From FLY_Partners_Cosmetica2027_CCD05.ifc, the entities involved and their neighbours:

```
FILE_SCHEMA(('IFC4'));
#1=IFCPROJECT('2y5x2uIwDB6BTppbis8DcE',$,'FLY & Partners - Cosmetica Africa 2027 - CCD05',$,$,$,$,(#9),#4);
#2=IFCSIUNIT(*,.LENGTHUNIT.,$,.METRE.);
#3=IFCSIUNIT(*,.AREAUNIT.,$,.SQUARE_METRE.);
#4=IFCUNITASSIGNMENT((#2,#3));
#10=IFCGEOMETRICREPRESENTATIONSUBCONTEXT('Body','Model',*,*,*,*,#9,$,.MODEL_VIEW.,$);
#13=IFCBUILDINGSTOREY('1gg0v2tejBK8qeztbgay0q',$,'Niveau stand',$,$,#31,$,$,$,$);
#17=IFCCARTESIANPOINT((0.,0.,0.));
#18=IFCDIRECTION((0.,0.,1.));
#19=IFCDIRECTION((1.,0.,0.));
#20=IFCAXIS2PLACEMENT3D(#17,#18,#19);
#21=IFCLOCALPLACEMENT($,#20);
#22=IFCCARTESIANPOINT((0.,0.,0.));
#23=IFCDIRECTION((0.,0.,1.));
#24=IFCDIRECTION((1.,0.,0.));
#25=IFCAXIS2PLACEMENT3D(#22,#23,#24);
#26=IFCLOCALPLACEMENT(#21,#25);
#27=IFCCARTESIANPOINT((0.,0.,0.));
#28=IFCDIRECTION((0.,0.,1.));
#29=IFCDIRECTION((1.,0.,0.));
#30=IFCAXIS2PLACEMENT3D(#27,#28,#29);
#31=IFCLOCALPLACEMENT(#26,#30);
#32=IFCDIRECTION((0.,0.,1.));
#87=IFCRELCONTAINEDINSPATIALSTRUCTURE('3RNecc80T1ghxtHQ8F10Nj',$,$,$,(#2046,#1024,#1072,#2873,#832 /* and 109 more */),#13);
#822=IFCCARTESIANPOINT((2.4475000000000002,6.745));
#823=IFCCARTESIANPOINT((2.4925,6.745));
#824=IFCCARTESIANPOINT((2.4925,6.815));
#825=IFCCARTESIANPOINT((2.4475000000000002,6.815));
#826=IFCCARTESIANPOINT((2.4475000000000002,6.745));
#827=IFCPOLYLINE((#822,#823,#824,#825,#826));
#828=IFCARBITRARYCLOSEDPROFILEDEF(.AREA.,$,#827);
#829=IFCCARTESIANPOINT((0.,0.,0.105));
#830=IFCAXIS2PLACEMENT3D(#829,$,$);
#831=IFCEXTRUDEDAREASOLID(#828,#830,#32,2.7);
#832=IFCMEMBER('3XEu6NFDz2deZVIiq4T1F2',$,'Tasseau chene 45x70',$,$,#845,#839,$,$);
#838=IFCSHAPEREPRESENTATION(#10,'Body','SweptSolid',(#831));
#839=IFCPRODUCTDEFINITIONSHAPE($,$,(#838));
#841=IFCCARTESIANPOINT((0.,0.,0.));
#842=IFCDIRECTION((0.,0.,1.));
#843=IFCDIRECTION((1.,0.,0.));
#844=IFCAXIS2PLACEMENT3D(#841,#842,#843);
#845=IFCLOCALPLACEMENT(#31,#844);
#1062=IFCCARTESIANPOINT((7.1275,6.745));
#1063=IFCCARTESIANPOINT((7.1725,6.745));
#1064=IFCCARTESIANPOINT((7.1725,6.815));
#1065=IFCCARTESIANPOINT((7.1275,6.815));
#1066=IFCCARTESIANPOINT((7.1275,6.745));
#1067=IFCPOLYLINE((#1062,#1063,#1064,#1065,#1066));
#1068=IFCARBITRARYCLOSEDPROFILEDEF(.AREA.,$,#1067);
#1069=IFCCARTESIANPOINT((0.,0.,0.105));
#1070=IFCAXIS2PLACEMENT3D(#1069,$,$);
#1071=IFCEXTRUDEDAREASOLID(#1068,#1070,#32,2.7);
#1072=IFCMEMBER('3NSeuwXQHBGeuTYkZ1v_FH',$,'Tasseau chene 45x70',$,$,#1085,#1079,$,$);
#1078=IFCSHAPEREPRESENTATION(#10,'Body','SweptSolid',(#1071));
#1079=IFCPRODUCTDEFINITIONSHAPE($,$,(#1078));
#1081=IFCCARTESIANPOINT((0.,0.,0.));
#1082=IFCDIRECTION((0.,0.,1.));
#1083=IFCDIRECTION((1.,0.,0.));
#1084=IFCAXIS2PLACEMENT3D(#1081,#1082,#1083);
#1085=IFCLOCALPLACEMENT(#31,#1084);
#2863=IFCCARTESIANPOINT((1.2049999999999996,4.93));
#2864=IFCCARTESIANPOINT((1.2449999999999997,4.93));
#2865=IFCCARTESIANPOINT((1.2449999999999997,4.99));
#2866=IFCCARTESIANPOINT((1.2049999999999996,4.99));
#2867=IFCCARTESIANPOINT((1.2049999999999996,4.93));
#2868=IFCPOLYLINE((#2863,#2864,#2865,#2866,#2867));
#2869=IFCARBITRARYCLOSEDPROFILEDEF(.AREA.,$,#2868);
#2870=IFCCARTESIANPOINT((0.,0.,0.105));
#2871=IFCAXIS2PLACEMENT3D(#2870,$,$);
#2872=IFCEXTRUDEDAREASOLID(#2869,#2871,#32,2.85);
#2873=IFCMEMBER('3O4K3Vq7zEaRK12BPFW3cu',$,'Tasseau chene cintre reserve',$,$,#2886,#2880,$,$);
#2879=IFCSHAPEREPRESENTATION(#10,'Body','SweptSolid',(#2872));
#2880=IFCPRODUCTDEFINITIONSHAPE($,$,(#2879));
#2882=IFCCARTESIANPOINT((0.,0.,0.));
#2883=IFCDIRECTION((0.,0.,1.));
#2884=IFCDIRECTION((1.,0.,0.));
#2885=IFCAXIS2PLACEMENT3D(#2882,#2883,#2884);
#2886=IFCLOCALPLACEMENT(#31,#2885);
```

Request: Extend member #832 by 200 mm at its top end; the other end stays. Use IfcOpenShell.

```python
import ifcopenshell
import ifcopenshell.util.representation
import ifcopenshell.util.unit

model = ifcopenshell.open("FLY_Partners_Cosmetica2027_CCD05.ifc")
unit_scale = ifcopenshell.util.unit.calculate_unit_scale(model)

member = model.by_guid("3XEu6NFDz2deZVIiq4T1F2")
change = 0.2 / unit_scale

# The extrusion runs towards the end named, so only its depth changes.
body = ifcopenshell.util.representation.get_representation(member, "Model", "Body")
solid = body.Items[0]
old_length = solid.Depth
solid.Depth += change

print(f"length {old_length:g} -> {solid.Depth:g}")

model.write("FLY_Partners_Cosmetica2027_CCD05_v2.ifc")
```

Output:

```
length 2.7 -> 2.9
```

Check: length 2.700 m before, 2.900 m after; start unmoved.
